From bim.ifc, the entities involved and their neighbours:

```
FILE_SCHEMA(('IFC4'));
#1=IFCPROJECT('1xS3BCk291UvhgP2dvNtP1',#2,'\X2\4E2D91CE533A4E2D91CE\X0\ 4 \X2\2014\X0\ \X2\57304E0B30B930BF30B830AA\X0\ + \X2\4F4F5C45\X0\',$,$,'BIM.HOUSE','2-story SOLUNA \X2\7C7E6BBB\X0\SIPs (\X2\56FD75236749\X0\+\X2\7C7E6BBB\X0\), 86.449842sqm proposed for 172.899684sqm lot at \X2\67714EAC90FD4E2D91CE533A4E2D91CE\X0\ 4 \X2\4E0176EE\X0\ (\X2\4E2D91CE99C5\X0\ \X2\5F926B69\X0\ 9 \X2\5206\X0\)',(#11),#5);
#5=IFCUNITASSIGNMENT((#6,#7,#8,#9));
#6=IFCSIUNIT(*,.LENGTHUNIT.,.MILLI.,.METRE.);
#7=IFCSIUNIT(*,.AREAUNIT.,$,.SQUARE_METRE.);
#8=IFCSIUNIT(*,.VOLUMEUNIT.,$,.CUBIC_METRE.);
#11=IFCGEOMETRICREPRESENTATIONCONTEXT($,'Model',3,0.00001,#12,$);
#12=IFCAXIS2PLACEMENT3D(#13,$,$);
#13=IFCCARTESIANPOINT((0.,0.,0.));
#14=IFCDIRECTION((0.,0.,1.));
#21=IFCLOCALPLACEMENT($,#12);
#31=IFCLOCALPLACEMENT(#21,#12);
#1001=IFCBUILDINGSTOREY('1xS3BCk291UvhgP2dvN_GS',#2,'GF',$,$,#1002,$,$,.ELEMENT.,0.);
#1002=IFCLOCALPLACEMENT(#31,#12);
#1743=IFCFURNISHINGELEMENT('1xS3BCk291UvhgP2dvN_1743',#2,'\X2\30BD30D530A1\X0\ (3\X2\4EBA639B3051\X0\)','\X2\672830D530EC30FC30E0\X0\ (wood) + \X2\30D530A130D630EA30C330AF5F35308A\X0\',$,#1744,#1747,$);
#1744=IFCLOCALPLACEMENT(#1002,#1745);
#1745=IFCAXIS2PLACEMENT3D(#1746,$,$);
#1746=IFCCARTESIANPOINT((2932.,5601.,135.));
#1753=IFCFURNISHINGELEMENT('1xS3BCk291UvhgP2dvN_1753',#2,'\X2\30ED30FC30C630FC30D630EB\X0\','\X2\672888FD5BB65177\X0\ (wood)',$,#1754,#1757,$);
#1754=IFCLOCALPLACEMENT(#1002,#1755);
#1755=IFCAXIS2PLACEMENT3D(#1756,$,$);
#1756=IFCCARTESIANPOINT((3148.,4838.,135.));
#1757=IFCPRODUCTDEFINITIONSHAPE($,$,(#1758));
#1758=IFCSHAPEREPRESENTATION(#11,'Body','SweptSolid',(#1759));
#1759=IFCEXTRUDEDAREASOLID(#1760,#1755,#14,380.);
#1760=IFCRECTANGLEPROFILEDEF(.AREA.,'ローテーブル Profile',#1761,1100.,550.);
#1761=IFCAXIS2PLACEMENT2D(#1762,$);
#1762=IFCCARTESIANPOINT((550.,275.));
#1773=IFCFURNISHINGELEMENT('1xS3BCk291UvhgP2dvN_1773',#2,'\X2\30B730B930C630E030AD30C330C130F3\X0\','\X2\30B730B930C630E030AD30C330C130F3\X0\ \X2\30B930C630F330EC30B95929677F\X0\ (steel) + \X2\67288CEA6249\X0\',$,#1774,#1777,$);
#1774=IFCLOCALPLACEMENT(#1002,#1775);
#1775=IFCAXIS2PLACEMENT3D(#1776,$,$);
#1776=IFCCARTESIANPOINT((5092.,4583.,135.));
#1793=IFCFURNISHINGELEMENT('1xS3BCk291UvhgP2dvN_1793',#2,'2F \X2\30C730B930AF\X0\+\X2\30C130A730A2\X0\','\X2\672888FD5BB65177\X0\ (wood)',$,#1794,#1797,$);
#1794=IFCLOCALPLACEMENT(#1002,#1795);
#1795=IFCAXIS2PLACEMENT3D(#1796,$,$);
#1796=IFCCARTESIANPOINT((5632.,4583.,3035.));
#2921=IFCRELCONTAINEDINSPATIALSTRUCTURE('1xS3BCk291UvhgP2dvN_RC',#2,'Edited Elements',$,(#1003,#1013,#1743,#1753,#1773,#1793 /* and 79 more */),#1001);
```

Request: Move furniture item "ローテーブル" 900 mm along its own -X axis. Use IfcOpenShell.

```python
import ifcopenshell
import ifcopenshell.api.geometry
import ifcopenshell.util.placement

model = ifcopenshell.open("bim.ifc")

item = model.by_guid("1xS3BCk291UvhgP2dvN_1753")
matrix = ifcopenshell.util.placement.get_local_placement(item.ObjectPlacement)
matrix[:3, 3] -= matrix[:3, 0] * 900.0
ifcopenshell.api.geometry.edit_object_placement(model, product=item, matrix=matrix, is_si=False)

print(ifcopenshell.util.placement.get_local_placement(item.ObjectPlacement).round(3) + 0.0)

model.write("bim-out.ifc")
```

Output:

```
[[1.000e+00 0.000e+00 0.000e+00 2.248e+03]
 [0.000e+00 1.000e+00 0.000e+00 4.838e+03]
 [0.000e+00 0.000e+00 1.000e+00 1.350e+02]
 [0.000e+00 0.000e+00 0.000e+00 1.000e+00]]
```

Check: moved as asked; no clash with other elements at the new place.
